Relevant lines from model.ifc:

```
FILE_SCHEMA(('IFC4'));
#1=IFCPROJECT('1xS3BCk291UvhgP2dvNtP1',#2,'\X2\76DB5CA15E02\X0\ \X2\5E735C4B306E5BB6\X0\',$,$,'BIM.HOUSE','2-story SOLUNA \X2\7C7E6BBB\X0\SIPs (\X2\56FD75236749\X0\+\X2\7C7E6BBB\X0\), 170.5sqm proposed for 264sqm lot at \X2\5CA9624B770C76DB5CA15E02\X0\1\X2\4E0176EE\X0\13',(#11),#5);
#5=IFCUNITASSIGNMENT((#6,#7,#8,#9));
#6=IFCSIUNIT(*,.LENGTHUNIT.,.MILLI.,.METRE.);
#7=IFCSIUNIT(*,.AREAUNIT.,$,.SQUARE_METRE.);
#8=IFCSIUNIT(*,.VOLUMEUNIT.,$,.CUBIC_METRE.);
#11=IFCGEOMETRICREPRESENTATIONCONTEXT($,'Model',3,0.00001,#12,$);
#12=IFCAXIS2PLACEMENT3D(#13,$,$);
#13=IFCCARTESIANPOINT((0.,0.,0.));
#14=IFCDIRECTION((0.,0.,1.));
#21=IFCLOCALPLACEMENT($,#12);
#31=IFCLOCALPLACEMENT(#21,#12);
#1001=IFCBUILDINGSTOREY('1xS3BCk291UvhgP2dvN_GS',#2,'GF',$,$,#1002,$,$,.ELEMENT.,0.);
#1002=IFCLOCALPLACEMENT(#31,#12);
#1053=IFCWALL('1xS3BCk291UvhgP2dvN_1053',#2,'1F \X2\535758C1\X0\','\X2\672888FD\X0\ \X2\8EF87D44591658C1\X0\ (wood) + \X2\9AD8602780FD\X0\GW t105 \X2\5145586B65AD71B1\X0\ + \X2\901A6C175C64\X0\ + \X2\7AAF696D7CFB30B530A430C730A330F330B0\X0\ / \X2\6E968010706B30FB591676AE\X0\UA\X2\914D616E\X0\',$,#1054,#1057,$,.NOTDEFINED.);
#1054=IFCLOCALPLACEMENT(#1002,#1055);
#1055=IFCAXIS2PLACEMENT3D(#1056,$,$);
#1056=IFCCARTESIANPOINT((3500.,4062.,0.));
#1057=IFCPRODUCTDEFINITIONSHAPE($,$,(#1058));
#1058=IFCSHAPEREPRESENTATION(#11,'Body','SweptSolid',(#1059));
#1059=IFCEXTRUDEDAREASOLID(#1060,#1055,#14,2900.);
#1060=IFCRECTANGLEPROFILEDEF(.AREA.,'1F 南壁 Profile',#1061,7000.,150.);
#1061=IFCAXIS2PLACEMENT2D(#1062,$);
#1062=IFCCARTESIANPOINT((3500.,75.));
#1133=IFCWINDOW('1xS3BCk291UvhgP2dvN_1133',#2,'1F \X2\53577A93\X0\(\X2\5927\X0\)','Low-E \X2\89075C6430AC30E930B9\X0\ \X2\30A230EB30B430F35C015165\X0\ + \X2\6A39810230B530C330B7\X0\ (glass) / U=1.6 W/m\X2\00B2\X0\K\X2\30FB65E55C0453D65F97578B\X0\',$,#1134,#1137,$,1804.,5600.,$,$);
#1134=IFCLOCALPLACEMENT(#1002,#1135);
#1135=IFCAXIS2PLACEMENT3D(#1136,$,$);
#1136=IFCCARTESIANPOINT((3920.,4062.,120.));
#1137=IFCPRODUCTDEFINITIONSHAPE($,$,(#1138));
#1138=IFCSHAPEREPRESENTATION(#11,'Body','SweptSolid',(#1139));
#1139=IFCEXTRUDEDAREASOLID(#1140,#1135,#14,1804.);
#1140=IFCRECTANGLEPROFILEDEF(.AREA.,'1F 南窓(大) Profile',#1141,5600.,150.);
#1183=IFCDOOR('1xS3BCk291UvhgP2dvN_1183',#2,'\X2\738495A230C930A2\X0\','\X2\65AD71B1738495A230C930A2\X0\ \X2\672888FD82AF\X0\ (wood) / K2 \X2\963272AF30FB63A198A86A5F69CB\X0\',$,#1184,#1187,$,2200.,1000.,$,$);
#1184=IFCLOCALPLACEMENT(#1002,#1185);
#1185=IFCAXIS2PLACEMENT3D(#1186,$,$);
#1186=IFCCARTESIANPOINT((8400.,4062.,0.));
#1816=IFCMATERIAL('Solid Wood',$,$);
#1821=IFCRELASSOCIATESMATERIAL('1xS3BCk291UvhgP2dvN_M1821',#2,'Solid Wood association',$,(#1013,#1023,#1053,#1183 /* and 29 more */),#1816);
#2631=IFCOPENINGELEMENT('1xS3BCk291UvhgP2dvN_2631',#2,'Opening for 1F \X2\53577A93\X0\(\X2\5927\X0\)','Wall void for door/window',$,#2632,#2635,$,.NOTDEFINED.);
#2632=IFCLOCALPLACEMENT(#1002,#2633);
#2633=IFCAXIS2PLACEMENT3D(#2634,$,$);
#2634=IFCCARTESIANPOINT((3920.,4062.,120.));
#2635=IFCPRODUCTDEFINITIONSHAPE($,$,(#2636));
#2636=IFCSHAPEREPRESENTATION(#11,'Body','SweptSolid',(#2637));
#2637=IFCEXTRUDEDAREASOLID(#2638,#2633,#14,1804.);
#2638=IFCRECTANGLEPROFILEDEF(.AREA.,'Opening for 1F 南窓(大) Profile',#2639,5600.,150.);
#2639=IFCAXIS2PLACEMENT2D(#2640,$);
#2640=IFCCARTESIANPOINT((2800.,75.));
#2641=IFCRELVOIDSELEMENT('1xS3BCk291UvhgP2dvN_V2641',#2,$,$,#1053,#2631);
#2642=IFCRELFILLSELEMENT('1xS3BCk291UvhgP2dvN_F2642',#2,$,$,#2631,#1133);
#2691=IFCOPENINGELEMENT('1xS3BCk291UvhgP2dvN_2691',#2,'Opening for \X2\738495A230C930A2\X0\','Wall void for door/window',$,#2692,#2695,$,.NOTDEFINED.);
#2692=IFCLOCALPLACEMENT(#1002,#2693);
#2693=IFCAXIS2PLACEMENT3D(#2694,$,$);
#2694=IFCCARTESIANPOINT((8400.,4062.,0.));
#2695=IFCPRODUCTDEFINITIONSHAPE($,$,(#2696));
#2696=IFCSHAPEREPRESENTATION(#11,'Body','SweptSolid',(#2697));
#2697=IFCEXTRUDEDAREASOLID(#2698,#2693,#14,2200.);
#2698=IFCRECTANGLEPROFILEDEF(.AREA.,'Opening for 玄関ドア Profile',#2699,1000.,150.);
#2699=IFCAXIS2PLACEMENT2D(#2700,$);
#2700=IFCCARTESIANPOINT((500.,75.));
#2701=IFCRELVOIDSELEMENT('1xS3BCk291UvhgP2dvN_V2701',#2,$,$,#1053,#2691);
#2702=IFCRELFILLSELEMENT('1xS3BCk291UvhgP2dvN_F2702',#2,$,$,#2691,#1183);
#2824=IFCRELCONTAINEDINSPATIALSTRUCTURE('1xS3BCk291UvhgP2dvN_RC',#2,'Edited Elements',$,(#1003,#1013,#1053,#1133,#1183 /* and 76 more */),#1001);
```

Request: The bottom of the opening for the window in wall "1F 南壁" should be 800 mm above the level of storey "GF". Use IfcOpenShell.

```python
import numpy as np
import ifcopenshell
import ifcopenshell.api.geometry
import ifcopenshell.geom
import ifcopenshell.util.element
import ifcopenshell.util.placement
import ifcopenshell.util.shape
import ifcopenshell.util.unit

model = ifcopenshell.open("model.ifc")
unit_scale = ifcopenshell.util.unit.calculate_unit_scale(model)

window = model.by_id(1133)
opening = window.FillsVoids[0].RelatingOpeningElement
storey = ifcopenshell.util.element.get_container(window, ifc_class="IfcBuildingStorey")
level = ifcopenshell.util.placement.get_local_placement(storey.ObjectPlacement)[2, 3]

# The opening's origin need not be at the sill, so measure its lowest point.
shape = ifcopenshell.geom.create_shape(ifcopenshell.geom.settings(), opening)
bottom = ifcopenshell.util.shape.get_shape_bottom_elevation(shape, shape.geometry) / unit_scale
dz = level + 800.0 - bottom

shift = np.array([0.0, 0.0, dz])
# The window is not placed relative to its opening, so move both.
for product in (opening, window):
    matrix = ifcopenshell.util.placement.get_local_placement(product.ObjectPlacement)
    matrix[:3, 3] += shift
    ifcopenshell.api.geometry.edit_object_placement(model, product=product, matrix=matrix, is_si=False)

print(f"moved by {dz * unit_scale:+.3f} m")

model.write("model_updated.ifc")
```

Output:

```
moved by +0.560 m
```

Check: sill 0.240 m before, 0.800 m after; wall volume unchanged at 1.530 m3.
